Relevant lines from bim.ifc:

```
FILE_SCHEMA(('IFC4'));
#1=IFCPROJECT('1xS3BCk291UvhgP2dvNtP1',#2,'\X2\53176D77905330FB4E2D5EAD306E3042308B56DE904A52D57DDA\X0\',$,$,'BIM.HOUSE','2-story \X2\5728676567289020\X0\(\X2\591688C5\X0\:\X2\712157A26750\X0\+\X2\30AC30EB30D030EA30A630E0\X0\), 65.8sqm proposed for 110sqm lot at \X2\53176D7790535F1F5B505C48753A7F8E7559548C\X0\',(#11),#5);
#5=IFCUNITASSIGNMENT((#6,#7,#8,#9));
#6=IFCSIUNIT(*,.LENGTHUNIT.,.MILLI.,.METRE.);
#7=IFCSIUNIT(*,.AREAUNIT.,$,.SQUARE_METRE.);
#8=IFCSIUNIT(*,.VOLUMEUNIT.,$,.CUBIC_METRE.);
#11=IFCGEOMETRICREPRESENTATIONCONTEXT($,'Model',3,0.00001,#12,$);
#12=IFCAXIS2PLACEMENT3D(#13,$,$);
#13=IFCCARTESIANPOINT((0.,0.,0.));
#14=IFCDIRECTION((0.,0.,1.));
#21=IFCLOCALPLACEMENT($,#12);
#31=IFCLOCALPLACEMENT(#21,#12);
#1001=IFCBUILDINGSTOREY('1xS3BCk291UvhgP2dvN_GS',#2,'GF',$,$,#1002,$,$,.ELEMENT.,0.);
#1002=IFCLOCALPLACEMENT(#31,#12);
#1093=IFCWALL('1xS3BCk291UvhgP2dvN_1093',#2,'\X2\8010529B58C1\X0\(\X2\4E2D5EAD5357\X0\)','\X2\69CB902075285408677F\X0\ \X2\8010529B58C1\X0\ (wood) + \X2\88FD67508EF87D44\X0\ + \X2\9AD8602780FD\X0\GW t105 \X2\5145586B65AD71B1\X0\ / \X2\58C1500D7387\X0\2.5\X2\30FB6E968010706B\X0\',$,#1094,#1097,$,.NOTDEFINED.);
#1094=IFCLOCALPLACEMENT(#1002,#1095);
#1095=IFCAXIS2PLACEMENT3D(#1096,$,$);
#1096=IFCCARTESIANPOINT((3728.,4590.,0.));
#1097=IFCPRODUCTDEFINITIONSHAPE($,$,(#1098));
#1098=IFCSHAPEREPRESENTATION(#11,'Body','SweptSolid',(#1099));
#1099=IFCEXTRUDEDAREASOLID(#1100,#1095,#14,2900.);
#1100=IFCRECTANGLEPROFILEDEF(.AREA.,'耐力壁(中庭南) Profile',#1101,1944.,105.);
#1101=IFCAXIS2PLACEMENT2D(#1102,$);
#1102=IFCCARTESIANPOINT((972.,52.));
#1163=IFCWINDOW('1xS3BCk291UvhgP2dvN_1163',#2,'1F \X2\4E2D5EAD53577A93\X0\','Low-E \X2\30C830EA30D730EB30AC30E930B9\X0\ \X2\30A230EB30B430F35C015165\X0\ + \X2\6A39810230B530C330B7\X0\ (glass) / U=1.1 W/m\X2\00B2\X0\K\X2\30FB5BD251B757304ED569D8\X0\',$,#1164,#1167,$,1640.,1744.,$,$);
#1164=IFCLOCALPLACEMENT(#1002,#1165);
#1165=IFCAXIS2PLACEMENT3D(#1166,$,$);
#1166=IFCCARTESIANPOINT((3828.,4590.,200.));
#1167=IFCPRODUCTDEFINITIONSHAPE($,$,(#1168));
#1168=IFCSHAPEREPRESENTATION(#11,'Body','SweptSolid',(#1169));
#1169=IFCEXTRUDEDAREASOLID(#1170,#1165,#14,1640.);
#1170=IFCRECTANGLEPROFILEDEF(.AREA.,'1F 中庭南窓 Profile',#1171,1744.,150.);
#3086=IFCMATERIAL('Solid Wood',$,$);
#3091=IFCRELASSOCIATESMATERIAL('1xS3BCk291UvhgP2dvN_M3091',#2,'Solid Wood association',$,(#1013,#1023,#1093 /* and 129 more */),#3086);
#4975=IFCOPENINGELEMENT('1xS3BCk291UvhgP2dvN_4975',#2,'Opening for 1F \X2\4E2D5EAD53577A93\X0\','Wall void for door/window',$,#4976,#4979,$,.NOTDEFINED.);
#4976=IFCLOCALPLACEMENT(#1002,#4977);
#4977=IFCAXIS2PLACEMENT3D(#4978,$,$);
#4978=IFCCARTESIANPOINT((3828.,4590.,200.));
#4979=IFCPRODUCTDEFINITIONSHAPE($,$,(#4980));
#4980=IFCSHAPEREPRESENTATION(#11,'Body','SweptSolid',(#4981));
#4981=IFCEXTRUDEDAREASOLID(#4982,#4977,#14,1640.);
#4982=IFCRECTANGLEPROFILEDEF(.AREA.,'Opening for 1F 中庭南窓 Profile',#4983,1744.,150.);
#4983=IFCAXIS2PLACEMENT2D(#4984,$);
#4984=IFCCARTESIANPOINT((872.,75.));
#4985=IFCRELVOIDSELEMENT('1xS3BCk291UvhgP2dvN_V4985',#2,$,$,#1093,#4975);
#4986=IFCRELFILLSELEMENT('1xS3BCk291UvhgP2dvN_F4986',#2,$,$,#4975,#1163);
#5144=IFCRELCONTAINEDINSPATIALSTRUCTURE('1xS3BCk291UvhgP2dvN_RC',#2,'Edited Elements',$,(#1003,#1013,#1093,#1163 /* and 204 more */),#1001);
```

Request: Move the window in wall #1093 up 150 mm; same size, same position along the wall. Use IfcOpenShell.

```python
import numpy as np
import ifcopenshell
import ifcopenshell.api.geometry
import ifcopenshell.util.placement
import ifcopenshell.util.unit

model = ifcopenshell.open("bim.ifc")
unit_scale = ifcopenshell.util.unit.calculate_unit_scale(model)

window = model.by_guid("1xS3BCk291UvhgP2dvN_1163")
opening = window.FillsVoids[0].RelatingOpeningElement
dz = 0.15 / unit_scale

shift = np.array([0.0, 0.0, dz])
# The window is not placed relative to its opening, so move both.
for product in (opening, window):
    matrix = ifcopenshell.util.placement.get_local_placement(product.ObjectPlacement)
    matrix[:3, 3] += shift
    ifcopenshell.api.geometry.edit_object_placement(model, product=product, matrix=matrix, is_si=False)

print(f"moved by {dz * unit_scale:+.3f} m")

model.write("bim_edited.ifc")
```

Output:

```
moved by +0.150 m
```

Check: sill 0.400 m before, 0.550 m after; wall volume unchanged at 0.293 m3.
